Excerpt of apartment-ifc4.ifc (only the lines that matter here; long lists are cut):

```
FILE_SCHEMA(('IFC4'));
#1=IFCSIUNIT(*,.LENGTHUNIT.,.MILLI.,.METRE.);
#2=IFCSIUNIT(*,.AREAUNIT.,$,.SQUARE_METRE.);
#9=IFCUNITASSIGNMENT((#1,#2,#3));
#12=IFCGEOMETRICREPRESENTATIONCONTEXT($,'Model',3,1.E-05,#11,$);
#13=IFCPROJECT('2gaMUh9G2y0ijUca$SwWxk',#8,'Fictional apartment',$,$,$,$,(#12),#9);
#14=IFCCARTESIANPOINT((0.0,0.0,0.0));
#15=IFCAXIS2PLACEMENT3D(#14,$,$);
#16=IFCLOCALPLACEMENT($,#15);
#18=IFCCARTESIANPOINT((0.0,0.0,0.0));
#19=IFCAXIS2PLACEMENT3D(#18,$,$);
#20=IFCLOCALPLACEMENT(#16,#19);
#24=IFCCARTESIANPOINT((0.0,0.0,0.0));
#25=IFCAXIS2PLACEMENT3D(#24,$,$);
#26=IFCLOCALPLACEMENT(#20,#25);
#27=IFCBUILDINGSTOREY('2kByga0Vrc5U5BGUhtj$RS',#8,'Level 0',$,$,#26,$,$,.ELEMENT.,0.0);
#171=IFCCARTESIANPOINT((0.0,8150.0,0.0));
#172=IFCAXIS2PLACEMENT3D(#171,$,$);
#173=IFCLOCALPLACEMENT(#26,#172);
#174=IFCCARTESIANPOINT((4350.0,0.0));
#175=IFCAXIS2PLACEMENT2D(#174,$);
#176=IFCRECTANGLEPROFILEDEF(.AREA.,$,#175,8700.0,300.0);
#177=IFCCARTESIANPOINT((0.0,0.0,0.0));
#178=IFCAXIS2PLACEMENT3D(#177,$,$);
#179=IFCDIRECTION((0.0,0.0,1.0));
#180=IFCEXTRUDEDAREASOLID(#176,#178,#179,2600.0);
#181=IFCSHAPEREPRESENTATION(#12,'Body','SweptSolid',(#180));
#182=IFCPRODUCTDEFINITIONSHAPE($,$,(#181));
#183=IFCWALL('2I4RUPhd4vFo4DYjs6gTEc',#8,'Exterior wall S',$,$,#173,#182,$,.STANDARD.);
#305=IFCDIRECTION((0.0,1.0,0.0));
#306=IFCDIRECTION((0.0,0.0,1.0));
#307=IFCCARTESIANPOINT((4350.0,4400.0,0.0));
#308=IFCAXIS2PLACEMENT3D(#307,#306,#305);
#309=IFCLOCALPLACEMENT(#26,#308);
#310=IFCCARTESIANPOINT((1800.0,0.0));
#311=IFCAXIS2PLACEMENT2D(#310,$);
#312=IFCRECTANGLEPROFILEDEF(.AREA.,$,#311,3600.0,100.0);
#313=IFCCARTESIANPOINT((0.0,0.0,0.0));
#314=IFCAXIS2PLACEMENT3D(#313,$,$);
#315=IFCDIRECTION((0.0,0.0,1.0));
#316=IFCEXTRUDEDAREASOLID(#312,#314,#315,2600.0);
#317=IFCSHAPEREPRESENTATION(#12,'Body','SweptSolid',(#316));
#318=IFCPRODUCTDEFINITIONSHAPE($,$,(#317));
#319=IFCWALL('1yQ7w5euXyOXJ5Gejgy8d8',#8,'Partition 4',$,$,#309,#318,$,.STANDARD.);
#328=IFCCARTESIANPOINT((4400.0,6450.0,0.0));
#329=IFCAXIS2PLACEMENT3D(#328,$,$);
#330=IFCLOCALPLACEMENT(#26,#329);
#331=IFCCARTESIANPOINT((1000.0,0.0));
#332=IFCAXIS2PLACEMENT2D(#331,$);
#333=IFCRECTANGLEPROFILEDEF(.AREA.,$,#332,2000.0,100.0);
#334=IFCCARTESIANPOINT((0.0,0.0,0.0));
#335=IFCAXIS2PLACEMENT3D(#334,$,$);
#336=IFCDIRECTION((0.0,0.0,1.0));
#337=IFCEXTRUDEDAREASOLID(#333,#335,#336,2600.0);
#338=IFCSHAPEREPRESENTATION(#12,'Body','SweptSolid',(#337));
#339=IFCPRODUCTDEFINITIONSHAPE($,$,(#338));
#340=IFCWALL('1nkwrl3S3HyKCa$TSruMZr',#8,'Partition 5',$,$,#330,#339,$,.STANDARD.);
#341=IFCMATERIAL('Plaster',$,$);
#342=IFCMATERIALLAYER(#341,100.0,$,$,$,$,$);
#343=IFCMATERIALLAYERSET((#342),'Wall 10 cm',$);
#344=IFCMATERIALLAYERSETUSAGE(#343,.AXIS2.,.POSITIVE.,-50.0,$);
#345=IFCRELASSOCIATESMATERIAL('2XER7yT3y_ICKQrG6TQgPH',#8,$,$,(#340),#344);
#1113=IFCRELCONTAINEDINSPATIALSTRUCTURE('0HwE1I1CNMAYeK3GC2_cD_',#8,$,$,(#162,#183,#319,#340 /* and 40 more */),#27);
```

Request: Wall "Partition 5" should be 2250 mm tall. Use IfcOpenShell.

```python
import ifcopenshell
import ifcopenshell.geom
import ifcopenshell.util.shape

model = ifcopenshell.open("apartment-ifc4.ifc")
settings = ifcopenshell.geom.settings()


def volume(element):
    """Net volume in cubic metres, openings subtracted."""
    shape = ifcopenshell.geom.create_shape(settings, element)
    return ifcopenshell.util.shape.get_volume(shape.geometry)


wall = model.by_guid("1nkwrl3S3HyKCa$TSruMZr")
before = volume(wall)

body = next(r for r in wall.Representation.Representations if r.RepresentationIdentifier == "Body")
solid = body.Items[0]
old_height = solid.Depth
solid.Depth = 2250.0
after = volume(wall)

print(f"height {old_height:g} -> {solid.Depth:g}, volume {before:.3f} -> {after:.3f} m3")

model.write("apartment-ifc4_rev.ifc")
```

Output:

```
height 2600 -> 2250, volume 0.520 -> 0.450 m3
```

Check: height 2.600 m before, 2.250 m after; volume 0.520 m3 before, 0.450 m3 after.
